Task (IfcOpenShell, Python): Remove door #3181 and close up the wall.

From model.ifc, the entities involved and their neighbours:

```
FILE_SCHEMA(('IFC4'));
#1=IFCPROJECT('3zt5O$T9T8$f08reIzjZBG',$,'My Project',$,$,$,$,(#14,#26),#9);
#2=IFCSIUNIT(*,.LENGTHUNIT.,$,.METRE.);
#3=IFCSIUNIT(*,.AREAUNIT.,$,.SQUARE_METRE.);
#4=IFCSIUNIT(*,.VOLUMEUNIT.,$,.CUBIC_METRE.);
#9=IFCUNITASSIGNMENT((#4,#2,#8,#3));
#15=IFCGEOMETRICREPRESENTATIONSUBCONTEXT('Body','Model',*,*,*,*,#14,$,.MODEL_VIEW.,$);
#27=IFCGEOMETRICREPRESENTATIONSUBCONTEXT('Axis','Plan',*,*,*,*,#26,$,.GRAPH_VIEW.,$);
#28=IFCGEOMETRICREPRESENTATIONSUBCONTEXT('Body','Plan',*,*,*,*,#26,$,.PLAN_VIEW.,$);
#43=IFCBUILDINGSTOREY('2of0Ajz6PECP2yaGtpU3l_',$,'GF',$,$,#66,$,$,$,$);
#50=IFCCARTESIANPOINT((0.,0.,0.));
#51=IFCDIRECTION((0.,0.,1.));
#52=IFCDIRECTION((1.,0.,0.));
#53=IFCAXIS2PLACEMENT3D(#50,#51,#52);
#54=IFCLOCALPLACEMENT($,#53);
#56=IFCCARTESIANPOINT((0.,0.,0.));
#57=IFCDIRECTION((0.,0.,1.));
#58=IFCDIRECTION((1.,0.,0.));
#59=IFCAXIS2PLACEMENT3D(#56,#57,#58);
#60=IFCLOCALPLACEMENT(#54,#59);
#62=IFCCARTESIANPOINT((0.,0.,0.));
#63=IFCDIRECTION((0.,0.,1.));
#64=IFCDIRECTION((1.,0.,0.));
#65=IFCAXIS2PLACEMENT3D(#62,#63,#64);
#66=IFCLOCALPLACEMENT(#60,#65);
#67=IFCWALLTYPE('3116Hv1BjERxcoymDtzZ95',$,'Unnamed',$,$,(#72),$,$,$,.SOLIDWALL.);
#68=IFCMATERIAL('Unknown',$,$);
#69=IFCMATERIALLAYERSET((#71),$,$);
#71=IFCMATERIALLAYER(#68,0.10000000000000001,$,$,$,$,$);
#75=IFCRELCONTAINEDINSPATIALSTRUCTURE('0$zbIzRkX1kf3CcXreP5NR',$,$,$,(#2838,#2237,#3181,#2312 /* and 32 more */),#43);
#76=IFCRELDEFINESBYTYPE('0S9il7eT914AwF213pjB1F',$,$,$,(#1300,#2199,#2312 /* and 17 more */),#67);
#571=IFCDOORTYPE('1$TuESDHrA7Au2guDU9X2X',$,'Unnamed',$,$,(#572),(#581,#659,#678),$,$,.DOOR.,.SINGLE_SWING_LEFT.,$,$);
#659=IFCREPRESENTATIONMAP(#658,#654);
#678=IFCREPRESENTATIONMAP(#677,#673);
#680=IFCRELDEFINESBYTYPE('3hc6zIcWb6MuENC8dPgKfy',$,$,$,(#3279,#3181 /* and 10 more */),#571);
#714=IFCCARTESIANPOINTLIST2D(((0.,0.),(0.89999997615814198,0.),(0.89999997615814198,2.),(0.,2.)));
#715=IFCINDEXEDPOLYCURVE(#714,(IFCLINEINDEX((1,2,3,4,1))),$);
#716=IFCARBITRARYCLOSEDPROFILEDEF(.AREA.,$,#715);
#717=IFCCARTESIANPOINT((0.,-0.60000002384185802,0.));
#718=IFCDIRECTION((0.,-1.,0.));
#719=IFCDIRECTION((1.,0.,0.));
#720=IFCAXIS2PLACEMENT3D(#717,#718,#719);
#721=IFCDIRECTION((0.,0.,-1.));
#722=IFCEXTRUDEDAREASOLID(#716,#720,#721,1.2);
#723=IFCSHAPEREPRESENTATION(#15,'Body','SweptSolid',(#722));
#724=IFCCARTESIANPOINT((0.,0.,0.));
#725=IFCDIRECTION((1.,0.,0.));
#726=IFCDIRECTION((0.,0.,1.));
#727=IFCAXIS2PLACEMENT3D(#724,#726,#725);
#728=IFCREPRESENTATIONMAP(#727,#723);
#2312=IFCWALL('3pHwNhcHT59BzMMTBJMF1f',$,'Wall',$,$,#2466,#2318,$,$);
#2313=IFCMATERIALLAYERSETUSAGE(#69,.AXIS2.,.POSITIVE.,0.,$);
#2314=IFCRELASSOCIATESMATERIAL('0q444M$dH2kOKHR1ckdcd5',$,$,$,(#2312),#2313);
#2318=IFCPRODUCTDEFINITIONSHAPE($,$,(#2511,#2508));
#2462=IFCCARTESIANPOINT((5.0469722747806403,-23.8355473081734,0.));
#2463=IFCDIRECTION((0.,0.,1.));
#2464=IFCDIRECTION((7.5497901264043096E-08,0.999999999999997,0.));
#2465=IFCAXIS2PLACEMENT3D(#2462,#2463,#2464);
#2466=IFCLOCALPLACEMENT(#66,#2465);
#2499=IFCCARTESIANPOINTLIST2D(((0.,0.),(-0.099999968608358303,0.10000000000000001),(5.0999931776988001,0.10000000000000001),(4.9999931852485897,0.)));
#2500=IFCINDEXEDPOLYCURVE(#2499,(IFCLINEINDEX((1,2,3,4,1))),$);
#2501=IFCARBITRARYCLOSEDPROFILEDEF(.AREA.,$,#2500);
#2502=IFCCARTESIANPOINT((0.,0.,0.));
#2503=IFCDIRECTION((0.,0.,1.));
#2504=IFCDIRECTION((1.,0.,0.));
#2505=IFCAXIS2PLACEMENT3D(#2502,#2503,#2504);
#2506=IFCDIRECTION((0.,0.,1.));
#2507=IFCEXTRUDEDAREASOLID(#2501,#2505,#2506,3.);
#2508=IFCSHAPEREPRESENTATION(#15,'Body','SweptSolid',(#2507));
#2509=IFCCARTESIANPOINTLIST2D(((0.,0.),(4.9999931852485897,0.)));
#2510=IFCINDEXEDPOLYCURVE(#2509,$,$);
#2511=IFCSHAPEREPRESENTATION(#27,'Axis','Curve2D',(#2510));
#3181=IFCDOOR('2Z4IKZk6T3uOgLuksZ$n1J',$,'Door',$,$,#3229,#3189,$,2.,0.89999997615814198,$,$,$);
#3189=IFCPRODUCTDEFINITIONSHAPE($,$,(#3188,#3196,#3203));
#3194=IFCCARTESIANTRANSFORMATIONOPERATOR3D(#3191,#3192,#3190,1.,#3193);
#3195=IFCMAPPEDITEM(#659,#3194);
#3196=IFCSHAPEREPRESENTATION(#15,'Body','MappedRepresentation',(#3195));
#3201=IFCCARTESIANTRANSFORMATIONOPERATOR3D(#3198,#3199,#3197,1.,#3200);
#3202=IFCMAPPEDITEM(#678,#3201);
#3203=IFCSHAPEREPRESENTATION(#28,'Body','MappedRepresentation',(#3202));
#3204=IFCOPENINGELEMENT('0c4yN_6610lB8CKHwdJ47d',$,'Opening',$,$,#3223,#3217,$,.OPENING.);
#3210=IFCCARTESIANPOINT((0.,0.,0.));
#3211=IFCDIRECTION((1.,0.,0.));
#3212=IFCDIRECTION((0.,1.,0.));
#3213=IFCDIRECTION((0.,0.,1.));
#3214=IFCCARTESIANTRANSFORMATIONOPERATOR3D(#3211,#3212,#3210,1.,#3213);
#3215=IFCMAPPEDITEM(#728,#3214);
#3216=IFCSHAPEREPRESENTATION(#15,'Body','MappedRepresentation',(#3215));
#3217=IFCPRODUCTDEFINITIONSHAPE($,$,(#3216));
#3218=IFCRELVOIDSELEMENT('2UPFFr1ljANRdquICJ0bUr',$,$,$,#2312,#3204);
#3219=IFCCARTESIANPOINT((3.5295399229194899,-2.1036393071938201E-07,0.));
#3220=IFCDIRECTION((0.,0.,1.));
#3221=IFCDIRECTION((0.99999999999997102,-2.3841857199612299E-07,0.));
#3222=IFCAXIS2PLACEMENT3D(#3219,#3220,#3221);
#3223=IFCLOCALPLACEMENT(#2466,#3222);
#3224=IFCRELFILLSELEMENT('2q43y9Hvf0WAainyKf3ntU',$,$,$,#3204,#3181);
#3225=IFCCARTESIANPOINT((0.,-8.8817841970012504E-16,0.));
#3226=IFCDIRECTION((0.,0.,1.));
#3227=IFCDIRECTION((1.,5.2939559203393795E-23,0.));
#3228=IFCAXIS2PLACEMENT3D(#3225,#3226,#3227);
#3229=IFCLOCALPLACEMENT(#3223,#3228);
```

```python
import ifcopenshell
import ifcopenshell.api.feature
import ifcopenshell.api.root
import ifcopenshell.geom
import ifcopenshell.util.shape

model = ifcopenshell.open("model.ifc")
settings = ifcopenshell.geom.settings()


def volume(element):
    """Net volume in cubic metres, openings subtracted."""
    shape = ifcopenshell.geom.create_shape(settings, element)
    return ifcopenshell.util.shape.get_volume(shape.geometry)


door = model.by_guid("2Z4IKZk6T3uOgLuksZ$n1J")
opening = door.FillsVoids[0].RelatingOpeningElement
wall = opening.VoidsElements[0].RelatingBuildingElement
before = volume(wall)

ifcopenshell.api.root.remove_product(model, product=door)
ifcopenshell.api.feature.remove_feature(model, feature=opening)

after = volume(wall)

print(f"wall volume {before:.3f} -> {after:.3f} m3")

model.write("model_edited.ifc")
```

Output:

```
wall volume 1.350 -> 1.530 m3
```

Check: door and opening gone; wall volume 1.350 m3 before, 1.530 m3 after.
